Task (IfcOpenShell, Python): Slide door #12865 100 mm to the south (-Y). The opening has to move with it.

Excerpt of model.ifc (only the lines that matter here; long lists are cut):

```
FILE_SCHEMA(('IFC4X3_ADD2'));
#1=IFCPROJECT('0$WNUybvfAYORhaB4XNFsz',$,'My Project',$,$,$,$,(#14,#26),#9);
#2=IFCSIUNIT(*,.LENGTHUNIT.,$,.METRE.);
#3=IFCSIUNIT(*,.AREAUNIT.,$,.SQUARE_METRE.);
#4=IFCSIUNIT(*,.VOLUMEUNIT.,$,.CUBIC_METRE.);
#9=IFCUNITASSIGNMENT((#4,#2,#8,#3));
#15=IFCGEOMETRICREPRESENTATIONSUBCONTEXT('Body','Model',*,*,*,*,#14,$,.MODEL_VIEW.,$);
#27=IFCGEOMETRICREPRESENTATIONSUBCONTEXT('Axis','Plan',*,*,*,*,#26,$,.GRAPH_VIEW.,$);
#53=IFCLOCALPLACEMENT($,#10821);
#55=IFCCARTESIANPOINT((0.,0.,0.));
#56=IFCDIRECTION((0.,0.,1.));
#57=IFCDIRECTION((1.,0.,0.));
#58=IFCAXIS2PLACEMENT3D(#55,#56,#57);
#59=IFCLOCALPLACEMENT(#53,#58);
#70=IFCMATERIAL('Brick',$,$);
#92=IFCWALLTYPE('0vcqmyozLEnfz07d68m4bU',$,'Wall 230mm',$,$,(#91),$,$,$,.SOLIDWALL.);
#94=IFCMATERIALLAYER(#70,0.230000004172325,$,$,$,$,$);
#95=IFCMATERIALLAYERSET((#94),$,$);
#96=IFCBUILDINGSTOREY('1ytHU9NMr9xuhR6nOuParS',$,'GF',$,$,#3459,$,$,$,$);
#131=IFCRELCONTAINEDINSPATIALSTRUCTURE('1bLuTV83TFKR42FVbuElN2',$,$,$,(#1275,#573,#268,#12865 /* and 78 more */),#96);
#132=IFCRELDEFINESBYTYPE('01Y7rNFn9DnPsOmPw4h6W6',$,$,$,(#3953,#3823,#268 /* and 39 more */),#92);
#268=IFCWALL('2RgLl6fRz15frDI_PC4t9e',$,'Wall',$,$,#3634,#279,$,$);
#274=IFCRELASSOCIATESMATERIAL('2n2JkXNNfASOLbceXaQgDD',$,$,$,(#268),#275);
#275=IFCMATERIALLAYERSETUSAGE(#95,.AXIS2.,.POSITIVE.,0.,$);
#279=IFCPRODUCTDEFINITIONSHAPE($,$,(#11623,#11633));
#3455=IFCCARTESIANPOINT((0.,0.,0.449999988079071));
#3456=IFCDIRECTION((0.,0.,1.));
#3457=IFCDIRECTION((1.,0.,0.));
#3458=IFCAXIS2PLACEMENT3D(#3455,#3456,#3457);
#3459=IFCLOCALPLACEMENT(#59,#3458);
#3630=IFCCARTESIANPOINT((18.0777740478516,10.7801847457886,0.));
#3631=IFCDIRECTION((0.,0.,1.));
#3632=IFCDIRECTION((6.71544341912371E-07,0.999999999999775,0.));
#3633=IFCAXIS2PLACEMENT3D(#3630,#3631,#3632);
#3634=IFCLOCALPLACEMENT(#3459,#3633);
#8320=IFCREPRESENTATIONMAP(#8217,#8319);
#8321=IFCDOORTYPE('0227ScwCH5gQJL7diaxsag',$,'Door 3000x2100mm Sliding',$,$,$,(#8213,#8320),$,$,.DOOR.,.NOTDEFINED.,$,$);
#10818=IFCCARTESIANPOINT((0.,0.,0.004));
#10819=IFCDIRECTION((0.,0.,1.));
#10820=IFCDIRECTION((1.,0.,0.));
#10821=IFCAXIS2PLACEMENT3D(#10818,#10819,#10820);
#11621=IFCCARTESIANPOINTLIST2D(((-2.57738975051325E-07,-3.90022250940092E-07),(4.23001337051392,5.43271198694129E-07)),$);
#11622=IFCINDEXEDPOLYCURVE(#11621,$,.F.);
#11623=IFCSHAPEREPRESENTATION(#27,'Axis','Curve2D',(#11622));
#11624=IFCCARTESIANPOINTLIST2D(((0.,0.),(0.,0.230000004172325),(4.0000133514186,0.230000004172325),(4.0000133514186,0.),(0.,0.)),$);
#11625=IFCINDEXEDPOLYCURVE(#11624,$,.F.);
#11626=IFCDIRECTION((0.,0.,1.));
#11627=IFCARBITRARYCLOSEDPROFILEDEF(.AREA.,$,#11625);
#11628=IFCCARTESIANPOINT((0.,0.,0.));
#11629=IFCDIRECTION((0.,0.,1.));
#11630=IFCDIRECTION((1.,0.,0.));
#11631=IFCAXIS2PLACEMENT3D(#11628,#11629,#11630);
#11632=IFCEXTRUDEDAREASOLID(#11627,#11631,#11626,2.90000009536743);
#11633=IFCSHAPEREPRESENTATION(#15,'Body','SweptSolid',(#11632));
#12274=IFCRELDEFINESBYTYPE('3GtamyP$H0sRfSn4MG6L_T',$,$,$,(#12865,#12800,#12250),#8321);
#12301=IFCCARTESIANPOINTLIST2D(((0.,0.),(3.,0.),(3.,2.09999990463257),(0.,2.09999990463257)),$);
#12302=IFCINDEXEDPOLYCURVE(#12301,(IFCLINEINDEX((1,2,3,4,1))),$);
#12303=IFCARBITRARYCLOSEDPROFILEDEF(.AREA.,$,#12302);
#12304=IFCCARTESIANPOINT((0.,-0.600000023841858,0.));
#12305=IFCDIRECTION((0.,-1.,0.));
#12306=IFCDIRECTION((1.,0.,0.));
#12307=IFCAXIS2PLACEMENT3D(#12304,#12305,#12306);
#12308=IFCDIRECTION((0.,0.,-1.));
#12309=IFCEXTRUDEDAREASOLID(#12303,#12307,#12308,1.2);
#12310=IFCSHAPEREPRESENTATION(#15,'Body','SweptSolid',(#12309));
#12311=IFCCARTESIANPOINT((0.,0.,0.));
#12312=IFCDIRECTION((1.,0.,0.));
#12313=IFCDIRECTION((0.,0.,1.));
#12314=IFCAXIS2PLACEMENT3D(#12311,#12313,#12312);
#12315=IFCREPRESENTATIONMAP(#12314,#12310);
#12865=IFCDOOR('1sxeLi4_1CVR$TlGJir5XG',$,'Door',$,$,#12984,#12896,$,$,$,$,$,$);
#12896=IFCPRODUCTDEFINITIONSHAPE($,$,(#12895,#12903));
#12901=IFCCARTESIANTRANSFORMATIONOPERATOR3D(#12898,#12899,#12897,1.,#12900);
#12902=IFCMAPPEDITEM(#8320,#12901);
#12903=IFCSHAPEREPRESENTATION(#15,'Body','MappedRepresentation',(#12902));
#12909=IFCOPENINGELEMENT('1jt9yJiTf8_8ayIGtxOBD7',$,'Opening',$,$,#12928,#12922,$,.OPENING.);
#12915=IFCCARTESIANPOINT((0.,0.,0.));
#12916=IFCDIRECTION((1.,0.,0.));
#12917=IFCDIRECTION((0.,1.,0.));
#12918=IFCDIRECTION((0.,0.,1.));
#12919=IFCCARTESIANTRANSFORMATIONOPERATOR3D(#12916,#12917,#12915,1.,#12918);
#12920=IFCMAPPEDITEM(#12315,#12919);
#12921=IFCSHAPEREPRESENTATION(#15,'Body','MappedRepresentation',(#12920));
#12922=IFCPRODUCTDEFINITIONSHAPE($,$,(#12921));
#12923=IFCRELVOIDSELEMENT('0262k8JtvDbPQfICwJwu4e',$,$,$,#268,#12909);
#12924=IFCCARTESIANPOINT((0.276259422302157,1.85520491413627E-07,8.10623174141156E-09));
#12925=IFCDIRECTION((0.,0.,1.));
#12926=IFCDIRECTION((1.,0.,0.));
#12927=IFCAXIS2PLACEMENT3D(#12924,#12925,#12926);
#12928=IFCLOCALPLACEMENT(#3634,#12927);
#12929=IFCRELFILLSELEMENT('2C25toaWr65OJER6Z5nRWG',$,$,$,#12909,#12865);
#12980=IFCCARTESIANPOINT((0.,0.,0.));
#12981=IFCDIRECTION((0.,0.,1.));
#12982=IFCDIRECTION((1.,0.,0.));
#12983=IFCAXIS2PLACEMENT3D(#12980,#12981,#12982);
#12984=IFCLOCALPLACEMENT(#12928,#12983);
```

```python
import ifcopenshell
import ifcopenshell.api.geometry
import ifcopenshell.util.placement
import ifcopenshell.util.unit

model = ifcopenshell.open("model.ifc")
unit_scale = ifcopenshell.util.unit.calculate_unit_scale(model)

door = model.by_guid("1sxeLi4_1CVR$TlGJir5XG")
opening = door.FillsVoids[0].RelatingOpeningElement
wall = opening.VoidsElements[0].RelatingBuildingElement

wall_matrix = ifcopenshell.util.placement.get_local_placement(wall.ObjectPlacement)
shift = wall_matrix[:3, 0] * -0.1 / unit_scale
before = ifcopenshell.util.placement.get_local_placement(door.ObjectPlacement)[:3, 3].copy()

# The door is placed relative to its opening, so it follows when the opening moves.
matrix = ifcopenshell.util.placement.get_local_placement(opening.ObjectPlacement)
matrix[:3, 3] += shift
ifcopenshell.api.geometry.edit_object_placement(
    model, product=opening, matrix=matrix, is_si=False, should_transform_children=True
)

after = ifcopenshell.util.placement.get_local_placement(door.ObjectPlacement)[:3, 3]
print("door moved by", (after - before).round(3) + 0.0)

model.write("model_v2.ifc")
```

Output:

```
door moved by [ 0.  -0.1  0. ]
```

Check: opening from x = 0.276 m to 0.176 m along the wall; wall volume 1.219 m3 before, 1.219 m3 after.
